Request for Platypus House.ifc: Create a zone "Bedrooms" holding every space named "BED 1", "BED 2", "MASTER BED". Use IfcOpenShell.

First a look at what the model holds.

```python
import ifcopenshell

model = ifcopenshell.open("Platypus House.ifc")
print(model.schema)
seen = {}
for space in model.by_type("IfcSpace"):
    seen[space.LongName] = seen.get(space.LongName, 0) + 1
for name, count in sorted(seen.items(), key=str):
    print(count, "x", name)
print("zones:", [z.Name for z in model.by_type("IfcZone")][:20])
```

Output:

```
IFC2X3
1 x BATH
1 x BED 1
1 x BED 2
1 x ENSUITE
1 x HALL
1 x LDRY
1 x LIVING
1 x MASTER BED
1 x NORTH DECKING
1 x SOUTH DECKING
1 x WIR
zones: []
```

```python
import ifcopenshell
import ifcopenshell.api.group
import ifcopenshell.api.root

model = ifcopenshell.open("Platypus House.ifc")

names = {"BED 1", "BED 2", "MASTER BED"}
spaces = [s for s in model.by_type("IfcSpace") if s.LongName in names]

zone = ifcopenshell.api.root.create_entity(model, ifc_class="IfcZone", name="Bedrooms")
ifcopenshell.api.group.assign_group(model, products=spaces, group=zone)
print(len(spaces), "spaces in", zone.Name)

model.write("Platypus House_edited.ifc")
```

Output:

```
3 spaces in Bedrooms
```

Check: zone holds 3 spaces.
